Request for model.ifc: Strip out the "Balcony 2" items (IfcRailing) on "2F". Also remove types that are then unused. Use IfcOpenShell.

First a look at what the model holds.

```python
import ifcopenshell
import ifcopenshell.util.element

model = ifcopenshell.open("model.ifc")
print(model.schema)
storey = next(s for s in model.by_type("IfcBuildingStorey") if s.Name == "2F")
railings = [e for e in ifcopenshell.util.element.get_decomposition(storey) if e.is_a("IfcRailing")]
seen = {}
for e in railings:
    element_type = ifcopenshell.util.element.get_type(e)
    name = element_type.Name if element_type not in (None, e) else None
    seen[name] = seen.get(name, 0) + 1
for name, count in sorted(seen.items(), key=str):
    print(count, "x", name)
```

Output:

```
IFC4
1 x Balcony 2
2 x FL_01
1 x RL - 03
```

```python
import ifcopenshell
import ifcopenshell.api.root
import ifcopenshell.util.element

model = ifcopenshell.open("model.ifc")

storey = next(s for s in model.by_type("IfcBuildingStorey") if s.Name == "2F")
railings = [e for e in ifcopenshell.util.element.get_decomposition(storey) if e.is_a("IfcRailing")]
targets = [e for e in railings if (t := ifcopenshell.util.element.get_type(e)) not in (None, e) and t.Name == "Balcony 2"]
types = {ifcopenshell.util.element.get_type(e) for e in targets} - {None, *targets}

for e in targets:
    ifcopenshell.api.root.remove_product(model, product=e)
print(len(targets), "removed")

unused = [t for t in types if not ifcopenshell.util.element.get_types(t)]
for t in unused:
    ifcopenshell.api.root.remove_product(model, product=t)
print(len(unused), "unused types removed")

model.write("model-out.ifc")
```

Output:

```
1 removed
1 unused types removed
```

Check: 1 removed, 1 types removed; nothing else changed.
